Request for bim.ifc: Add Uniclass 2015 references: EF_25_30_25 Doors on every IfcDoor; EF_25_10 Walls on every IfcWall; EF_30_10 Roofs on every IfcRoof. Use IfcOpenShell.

First a look at what the model holds.

```python
import ifcopenshell

model = ifcopenshell.open("bim.ifc")
print(model.schema)
print("classifications:", [c.Name for c in model.by_type("IfcClassification")])
for ifc_class in ("IfcDoor", "IfcRoof", "IfcStair", "IfcWall", "IfcWindow"):
    print(ifc_class, len(model.by_type(ifc_class)))
```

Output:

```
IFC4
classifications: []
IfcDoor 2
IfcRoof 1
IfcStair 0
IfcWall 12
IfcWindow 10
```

```python
import ifcopenshell
import ifcopenshell.api.classification

model = ifcopenshell.open("bim.ifc")

system = ifcopenshell.api.classification.add_classification(model, classification="Uniclass 2015")

codes = {
    "IfcDoor": ("EF_25_30_25", "Doors"),
    "IfcWall": ("EF_25_10", "Walls"),
    "IfcRoof": ("EF_30_10", "Roofs"),
}
for ifc_class, (code, name) in codes.items():
    products = model.by_type(ifc_class)
    ifcopenshell.api.classification.add_reference(
        model, products=products, classification=system, identification=code, name=name
    )
    print(code, len(products))

model.write("bim_updated.ifc")
```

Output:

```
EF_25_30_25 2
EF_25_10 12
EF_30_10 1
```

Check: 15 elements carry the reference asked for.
